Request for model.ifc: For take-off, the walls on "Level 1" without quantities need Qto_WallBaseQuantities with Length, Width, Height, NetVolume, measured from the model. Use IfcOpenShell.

First a look at what the model holds.

```python
import ifcopenshell
import ifcopenshell.util.element
import ifcopenshell.util.unit

model = ifcopenshell.open("model.ifc")
print(model.schema)
for unit_type in ("LENGTHUNIT", "AREAUNIT", "VOLUMEUNIT"):
    print(unit_type, ifcopenshell.util.unit.calculate_unit_scale(model, unit_type))
storey = next(s for s in model.by_type("IfcBuildingStorey") if s.Name == "Level 1")
walls = [e for e in ifcopenshell.util.element.get_decomposition(storey) if e.is_a("IfcWall")]
for e in sorted(walls, key=lambda e: e.id()):
    print(e.id(), e.is_a(), e.Name, list(ifcopenshell.util.element.get_psets(e, qtos_only=True)), sep=" | ")
```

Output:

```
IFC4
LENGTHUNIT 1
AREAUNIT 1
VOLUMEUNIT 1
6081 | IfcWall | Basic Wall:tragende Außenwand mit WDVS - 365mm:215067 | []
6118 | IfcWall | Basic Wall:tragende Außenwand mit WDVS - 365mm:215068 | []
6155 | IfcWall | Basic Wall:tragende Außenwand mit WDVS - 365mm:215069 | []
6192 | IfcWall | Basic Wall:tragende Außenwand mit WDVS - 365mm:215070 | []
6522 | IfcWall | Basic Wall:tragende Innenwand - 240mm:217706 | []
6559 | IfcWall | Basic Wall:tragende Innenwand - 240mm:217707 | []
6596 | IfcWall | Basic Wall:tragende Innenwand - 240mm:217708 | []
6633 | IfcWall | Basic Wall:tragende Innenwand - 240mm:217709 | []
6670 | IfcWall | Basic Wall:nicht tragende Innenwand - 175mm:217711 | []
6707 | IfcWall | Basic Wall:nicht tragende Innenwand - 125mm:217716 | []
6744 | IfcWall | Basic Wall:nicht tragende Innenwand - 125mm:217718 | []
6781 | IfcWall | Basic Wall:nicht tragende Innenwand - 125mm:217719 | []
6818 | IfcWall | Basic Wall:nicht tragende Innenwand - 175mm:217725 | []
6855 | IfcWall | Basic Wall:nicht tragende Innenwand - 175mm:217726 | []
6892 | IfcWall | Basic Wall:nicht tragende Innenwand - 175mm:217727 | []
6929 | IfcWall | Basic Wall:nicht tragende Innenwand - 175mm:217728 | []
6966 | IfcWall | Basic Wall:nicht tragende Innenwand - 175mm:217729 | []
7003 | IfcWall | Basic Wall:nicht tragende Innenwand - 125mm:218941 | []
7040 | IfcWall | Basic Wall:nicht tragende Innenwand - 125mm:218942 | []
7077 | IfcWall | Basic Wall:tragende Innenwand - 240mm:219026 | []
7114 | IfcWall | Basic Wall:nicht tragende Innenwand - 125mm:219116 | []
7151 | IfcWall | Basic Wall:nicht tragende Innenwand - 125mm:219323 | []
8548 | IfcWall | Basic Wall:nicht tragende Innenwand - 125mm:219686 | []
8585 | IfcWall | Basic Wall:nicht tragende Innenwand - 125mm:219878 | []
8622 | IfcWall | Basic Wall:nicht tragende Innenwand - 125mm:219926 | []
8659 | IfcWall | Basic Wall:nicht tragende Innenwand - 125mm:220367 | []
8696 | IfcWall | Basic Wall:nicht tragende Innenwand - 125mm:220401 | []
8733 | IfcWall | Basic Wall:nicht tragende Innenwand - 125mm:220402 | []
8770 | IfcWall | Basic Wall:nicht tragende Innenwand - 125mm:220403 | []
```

```python
import ifcopenshell
import ifcopenshell.api.pset
import ifcopenshell.geom
import ifcopenshell.util.element
import ifcopenshell.util.shape
import ifcopenshell.util.unit

model = ifcopenshell.open("model.ifc")
unit_scale = ifcopenshell.util.unit.calculate_unit_scale(model)
volume_scale = ifcopenshell.util.unit.calculate_unit_scale(model, "VOLUMEUNIT")
settings = ifcopenshell.geom.settings()

storey = next(s for s in model.by_type("IfcBuildingStorey") if s.Name == "Level 1")
walls = [e for e in ifcopenshell.util.element.get_decomposition(storey) if e.is_a("IfcWall")]

for e in sorted(walls, key=lambda e: e.id()):
    if ifcopenshell.util.element.get_psets(e, qtos_only=True, should_inherit=False):
        continue
    # Geometry comes back in metres, in the element's own axes.
    shape = ifcopenshell.geom.create_shape(settings, e)
    values = {
        "Length": ifcopenshell.util.shape.get_x(shape.geometry) / unit_scale,
        "Width": ifcopenshell.util.shape.get_y(shape.geometry) / unit_scale,
        "Height": ifcopenshell.util.shape.get_z(shape.geometry) / unit_scale,
        "NetVolume": ifcopenshell.util.shape.get_volume(shape.geometry) / volume_scale,
    }
    qto = ifcopenshell.api.pset.add_qto(model, product=e, name="Qto_WallBaseQuantities")
    ifcopenshell.api.pset.edit_qto(model, qto=qto, properties=values)
    print(e.id(), {k: round(v, 3) for k, v in values.items()})

model.write("model_rev.ifc")
```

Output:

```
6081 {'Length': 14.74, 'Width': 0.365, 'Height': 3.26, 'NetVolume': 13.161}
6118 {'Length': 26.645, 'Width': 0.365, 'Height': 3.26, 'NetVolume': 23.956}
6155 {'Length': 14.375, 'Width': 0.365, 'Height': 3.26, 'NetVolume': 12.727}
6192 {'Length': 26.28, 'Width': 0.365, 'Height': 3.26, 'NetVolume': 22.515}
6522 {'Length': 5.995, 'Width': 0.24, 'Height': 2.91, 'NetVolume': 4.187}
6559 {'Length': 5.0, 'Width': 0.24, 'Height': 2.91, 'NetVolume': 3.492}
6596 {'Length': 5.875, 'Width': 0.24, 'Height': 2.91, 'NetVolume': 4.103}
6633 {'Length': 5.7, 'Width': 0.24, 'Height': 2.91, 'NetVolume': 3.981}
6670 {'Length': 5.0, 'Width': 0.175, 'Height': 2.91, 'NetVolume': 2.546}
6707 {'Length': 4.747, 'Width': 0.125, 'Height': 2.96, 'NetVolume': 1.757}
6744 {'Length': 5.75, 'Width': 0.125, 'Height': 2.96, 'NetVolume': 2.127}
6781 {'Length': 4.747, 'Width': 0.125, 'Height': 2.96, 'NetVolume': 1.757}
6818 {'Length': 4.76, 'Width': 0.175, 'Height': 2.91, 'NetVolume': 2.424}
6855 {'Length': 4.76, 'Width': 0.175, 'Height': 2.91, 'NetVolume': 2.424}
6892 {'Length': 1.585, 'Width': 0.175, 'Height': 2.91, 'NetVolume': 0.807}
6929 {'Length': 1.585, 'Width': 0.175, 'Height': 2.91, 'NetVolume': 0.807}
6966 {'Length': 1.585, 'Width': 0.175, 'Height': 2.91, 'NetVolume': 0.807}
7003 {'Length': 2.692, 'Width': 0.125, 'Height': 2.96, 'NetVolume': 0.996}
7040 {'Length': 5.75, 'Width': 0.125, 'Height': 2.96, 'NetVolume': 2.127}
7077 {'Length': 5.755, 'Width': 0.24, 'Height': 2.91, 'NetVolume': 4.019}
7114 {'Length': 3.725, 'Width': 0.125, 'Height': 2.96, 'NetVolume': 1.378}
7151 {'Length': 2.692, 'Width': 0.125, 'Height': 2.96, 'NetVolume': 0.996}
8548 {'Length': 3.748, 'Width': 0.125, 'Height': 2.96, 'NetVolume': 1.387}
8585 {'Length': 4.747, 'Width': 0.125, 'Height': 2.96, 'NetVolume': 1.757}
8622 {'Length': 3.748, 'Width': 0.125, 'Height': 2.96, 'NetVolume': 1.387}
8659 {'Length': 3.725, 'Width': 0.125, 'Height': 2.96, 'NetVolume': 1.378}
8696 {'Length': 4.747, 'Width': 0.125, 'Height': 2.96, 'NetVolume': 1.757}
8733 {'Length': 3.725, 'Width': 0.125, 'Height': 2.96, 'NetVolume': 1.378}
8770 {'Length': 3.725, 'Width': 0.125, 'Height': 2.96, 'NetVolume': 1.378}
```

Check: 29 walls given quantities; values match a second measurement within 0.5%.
